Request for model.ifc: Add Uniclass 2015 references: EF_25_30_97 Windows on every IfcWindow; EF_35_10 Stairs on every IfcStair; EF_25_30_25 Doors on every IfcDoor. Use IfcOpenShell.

First a look at what the model holds.

```python
import ifcopenshell

model = ifcopenshell.open("model.ifc")
print(model.schema)
print("classifications:", [c.Name for c in model.by_type("IfcClassification")])
for ifc_class in ("IfcDoor", "IfcRoof", "IfcStair", "IfcWall", "IfcWindow"):
    print(ifc_class, len(model.by_type(ifc_class)))
```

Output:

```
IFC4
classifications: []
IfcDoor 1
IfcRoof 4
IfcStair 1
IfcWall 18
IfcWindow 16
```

```python
import ifcopenshell
import ifcopenshell.api.classification

model = ifcopenshell.open("model.ifc")

system = ifcopenshell.api.classification.add_classification(model, classification="Uniclass 2015")

codes = {
    "IfcWindow": ("EF_25_30_97", "Windows"),
    "IfcStair": ("EF_35_10", "Stairs"),
    "IfcDoor": ("EF_25_30_25", "Doors"),
}
for ifc_class, (code, name) in codes.items():
    products = model.by_type(ifc_class)
    ifcopenshell.api.classification.add_reference(
        model, products=products, classification=system, identification=code, name=name
    )
    print(code, len(products))

model.write("model_rev.ifc")
```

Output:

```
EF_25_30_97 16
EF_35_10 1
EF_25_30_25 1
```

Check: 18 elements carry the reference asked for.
